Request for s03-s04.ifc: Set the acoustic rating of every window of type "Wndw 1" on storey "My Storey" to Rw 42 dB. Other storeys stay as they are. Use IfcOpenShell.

First a look at what the model holds.

```python
import ifcopenshell
import ifcopenshell.util.element

model = ifcopenshell.open("s03-s04.ifc")
print(model.schema)
storey = next(s for s in model.by_type("IfcBuildingStorey") if s.Name == "My Storey")
windows = [e for e in ifcopenshell.util.element.get_decomposition(storey) if e.is_a("IfcWindow")]
seen = {}
for e in windows:
    element_type = ifcopenshell.util.element.get_type(e)
    key = (element_type.Name if element_type != e and element_type else None, ifcopenshell.util.element.get_pset(e, "Pset_WindowCommon", "AcousticRating"))
    seen[key] = seen.get(key, 0) + 1
for (name, value), count in sorted(seen.items(), key=str):
    print(count, "x", name, "|", value)
```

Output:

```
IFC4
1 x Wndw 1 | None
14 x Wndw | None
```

```python
import ifcopenshell
import ifcopenshell.api.pset
import ifcopenshell.util.element

model = ifcopenshell.open("s03-s04.ifc")

storey = next(s for s in model.by_type("IfcBuildingStorey") if s.Name == "My Storey")
windows = [e for e in ifcopenshell.util.element.get_decomposition(storey) if e.is_a("IfcWindow")]

count = 0
for e in windows:
    element_type = ifcopenshell.util.element.get_type(e)
    if element_type in (None, e) or element_type.Name != "Wndw 1":
        continue
    # add_pset returns the element's existing set when there is one.
    pset = ifcopenshell.api.pset.add_pset(model, product=e, name="Pset_WindowCommon")
    ifcopenshell.api.pset.edit_pset(model, pset=pset, properties={"AcousticRating": "Rw 42 dB"})
    count += 1

print(count, "windows updated")

model.write("s03-s04_rev.ifc")
```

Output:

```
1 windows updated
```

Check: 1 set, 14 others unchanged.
